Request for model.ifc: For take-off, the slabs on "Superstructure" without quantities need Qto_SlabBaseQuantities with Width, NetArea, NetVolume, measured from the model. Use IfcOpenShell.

First a look at what the model holds.

```python
import ifcopenshell
import ifcopenshell.util.element
import ifcopenshell.util.unit

model = ifcopenshell.open("model.ifc")
print(model.schema)
for unit_type in ("LENGTHUNIT", "AREAUNIT", "VOLUMEUNIT"):
    print(unit_type, ifcopenshell.util.unit.calculate_unit_scale(model, unit_type))
storey = next(s for s in model.by_type("IfcBuildingStorey") if s.Name == "Superstructure")
slabs = [e for e in ifcopenshell.util.element.get_decomposition(storey) if e.is_a("IfcSlab")]
for e in sorted(slabs, key=lambda e: e.id()):
    print(e.id(), e.is_a(), e.Name, list(ifcopenshell.util.element.get_psets(e, qtos_only=True)), sep=" | ")
```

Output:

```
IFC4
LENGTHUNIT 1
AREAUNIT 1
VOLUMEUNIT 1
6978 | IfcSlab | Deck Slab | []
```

```python
import ifcopenshell
import ifcopenshell.api.pset
import ifcopenshell.geom
import ifcopenshell.util.element
import ifcopenshell.util.shape
import ifcopenshell.util.unit

model = ifcopenshell.open("model.ifc")
unit_scale = ifcopenshell.util.unit.calculate_unit_scale(model)
area_scale = ifcopenshell.util.unit.calculate_unit_scale(model, "AREAUNIT")
volume_scale = ifcopenshell.util.unit.calculate_unit_scale(model, "VOLUMEUNIT")
settings = ifcopenshell.geom.settings()

storey = next(s for s in model.by_type("IfcBuildingStorey") if s.Name == "Superstructure")
slabs = [e for e in ifcopenshell.util.element.get_decomposition(storey) if e.is_a("IfcSlab")]

for e in sorted(slabs, key=lambda e: e.id()):
    if ifcopenshell.util.element.get_psets(e, qtos_only=True, should_inherit=False):
        continue
    # Geometry comes back in metres, in the element's own axes.
    shape = ifcopenshell.geom.create_shape(settings, e)
    values = {
        "Width": ifcopenshell.util.shape.get_z(shape.geometry) / unit_scale,
        "NetArea": ifcopenshell.util.shape.get_footprint_area(shape.geometry) / area_scale,
        "NetVolume": ifcopenshell.util.shape.get_volume(shape.geometry) / volume_scale,
    }
    qto = ifcopenshell.api.pset.add_qto(model, product=e, name="Qto_SlabBaseQuantities")
    ifcopenshell.api.pset.edit_qto(model, qto=qto, properties=values)
    print(e.id(), {k: round(v, 3) for k, v in values.items()})

model.write("model_rev.ifc")
```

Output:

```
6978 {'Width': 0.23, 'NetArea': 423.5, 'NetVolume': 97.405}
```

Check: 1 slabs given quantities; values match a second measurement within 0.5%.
